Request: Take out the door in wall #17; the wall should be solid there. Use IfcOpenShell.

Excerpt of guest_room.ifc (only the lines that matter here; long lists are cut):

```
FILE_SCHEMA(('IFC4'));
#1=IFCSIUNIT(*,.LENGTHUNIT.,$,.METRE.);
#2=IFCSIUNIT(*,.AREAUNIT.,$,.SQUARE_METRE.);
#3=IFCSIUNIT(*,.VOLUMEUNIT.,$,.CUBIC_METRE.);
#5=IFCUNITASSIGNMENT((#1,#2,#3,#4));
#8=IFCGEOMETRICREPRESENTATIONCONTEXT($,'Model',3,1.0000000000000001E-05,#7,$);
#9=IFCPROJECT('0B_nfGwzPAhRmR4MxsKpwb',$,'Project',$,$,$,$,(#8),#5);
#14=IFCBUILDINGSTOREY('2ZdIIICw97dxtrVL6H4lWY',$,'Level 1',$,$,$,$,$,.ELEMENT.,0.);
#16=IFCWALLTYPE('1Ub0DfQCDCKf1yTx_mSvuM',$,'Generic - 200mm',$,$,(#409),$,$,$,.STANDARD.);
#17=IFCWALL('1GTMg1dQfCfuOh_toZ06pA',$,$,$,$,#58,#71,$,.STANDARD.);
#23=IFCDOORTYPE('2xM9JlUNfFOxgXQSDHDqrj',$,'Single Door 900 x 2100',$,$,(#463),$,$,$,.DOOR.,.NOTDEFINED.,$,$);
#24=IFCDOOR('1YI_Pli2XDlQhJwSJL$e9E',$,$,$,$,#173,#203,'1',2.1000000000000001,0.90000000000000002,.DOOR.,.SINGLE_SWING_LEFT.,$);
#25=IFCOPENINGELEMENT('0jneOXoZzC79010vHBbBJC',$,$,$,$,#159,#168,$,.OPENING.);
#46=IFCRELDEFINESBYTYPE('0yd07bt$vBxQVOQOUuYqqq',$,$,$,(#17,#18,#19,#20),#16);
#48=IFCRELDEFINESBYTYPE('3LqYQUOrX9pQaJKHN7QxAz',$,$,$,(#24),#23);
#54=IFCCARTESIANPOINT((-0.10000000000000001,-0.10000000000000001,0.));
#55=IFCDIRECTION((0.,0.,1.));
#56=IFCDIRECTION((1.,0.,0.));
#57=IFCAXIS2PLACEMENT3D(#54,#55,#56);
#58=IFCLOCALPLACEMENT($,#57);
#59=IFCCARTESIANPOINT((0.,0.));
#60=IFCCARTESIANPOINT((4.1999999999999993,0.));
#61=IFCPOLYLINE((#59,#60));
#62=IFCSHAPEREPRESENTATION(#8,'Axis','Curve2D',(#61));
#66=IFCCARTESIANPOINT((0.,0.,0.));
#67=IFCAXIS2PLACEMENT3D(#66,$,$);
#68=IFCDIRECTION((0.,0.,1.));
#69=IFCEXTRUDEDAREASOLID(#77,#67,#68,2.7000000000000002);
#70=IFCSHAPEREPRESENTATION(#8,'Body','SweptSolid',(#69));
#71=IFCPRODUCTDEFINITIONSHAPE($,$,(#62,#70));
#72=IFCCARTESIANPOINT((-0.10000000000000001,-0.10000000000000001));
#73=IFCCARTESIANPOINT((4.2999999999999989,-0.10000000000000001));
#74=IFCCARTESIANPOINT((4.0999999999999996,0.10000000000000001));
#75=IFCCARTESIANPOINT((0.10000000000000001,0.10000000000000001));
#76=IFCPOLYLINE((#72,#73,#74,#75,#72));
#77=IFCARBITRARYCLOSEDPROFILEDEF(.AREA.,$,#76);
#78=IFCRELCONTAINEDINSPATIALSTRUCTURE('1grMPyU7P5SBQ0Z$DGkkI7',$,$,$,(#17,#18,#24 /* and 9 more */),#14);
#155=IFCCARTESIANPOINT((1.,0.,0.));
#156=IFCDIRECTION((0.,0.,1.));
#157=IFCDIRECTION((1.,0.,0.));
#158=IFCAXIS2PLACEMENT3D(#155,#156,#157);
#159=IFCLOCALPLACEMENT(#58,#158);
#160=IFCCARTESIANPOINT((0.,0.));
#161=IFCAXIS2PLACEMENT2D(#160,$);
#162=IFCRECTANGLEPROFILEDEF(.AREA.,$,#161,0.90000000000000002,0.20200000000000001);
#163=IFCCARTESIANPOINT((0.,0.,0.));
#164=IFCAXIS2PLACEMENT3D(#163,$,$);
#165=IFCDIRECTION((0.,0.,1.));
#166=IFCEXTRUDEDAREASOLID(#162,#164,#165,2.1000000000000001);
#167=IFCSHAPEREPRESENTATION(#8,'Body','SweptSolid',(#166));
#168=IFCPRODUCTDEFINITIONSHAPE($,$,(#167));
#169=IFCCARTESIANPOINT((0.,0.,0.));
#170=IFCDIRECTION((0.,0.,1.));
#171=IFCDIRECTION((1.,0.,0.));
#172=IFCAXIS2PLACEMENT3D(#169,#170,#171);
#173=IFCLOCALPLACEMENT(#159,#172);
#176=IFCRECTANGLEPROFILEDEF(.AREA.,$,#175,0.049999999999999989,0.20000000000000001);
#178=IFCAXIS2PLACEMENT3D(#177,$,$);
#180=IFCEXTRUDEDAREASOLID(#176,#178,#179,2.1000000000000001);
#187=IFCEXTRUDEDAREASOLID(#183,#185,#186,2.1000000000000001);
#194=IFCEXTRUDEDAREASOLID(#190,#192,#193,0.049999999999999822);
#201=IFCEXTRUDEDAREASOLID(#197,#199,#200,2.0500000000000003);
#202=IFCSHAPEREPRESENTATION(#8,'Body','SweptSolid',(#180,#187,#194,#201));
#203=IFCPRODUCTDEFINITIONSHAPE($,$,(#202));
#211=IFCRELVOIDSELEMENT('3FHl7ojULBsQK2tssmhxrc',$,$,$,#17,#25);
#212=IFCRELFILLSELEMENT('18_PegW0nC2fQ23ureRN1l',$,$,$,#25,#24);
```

```python
import ifcopenshell
import ifcopenshell.api.feature
import ifcopenshell.api.root
import ifcopenshell.geom
import ifcopenshell.util.shape

model = ifcopenshell.open("guest_room.ifc")
settings = ifcopenshell.geom.settings()


def volume(element):
    """Net volume in cubic metres, openings subtracted."""
    shape = ifcopenshell.geom.create_shape(settings, element)
    return ifcopenshell.util.shape.get_volume(shape.geometry)


door = model.by_guid("1YI_Pli2XDlQhJwSJL$e9E")
opening = door.FillsVoids[0].RelatingOpeningElement
wall = opening.VoidsElements[0].RelatingBuildingElement
before = volume(wall)

ifcopenshell.api.root.remove_product(model, product=door)
ifcopenshell.api.feature.remove_feature(model, feature=opening)

after = volume(wall)

print(f"wall volume {before:.3f} -> {after:.3f} m3")

model.write("guest_room-out.ifc")
```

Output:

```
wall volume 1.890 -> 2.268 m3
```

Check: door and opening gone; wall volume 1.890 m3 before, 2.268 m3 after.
